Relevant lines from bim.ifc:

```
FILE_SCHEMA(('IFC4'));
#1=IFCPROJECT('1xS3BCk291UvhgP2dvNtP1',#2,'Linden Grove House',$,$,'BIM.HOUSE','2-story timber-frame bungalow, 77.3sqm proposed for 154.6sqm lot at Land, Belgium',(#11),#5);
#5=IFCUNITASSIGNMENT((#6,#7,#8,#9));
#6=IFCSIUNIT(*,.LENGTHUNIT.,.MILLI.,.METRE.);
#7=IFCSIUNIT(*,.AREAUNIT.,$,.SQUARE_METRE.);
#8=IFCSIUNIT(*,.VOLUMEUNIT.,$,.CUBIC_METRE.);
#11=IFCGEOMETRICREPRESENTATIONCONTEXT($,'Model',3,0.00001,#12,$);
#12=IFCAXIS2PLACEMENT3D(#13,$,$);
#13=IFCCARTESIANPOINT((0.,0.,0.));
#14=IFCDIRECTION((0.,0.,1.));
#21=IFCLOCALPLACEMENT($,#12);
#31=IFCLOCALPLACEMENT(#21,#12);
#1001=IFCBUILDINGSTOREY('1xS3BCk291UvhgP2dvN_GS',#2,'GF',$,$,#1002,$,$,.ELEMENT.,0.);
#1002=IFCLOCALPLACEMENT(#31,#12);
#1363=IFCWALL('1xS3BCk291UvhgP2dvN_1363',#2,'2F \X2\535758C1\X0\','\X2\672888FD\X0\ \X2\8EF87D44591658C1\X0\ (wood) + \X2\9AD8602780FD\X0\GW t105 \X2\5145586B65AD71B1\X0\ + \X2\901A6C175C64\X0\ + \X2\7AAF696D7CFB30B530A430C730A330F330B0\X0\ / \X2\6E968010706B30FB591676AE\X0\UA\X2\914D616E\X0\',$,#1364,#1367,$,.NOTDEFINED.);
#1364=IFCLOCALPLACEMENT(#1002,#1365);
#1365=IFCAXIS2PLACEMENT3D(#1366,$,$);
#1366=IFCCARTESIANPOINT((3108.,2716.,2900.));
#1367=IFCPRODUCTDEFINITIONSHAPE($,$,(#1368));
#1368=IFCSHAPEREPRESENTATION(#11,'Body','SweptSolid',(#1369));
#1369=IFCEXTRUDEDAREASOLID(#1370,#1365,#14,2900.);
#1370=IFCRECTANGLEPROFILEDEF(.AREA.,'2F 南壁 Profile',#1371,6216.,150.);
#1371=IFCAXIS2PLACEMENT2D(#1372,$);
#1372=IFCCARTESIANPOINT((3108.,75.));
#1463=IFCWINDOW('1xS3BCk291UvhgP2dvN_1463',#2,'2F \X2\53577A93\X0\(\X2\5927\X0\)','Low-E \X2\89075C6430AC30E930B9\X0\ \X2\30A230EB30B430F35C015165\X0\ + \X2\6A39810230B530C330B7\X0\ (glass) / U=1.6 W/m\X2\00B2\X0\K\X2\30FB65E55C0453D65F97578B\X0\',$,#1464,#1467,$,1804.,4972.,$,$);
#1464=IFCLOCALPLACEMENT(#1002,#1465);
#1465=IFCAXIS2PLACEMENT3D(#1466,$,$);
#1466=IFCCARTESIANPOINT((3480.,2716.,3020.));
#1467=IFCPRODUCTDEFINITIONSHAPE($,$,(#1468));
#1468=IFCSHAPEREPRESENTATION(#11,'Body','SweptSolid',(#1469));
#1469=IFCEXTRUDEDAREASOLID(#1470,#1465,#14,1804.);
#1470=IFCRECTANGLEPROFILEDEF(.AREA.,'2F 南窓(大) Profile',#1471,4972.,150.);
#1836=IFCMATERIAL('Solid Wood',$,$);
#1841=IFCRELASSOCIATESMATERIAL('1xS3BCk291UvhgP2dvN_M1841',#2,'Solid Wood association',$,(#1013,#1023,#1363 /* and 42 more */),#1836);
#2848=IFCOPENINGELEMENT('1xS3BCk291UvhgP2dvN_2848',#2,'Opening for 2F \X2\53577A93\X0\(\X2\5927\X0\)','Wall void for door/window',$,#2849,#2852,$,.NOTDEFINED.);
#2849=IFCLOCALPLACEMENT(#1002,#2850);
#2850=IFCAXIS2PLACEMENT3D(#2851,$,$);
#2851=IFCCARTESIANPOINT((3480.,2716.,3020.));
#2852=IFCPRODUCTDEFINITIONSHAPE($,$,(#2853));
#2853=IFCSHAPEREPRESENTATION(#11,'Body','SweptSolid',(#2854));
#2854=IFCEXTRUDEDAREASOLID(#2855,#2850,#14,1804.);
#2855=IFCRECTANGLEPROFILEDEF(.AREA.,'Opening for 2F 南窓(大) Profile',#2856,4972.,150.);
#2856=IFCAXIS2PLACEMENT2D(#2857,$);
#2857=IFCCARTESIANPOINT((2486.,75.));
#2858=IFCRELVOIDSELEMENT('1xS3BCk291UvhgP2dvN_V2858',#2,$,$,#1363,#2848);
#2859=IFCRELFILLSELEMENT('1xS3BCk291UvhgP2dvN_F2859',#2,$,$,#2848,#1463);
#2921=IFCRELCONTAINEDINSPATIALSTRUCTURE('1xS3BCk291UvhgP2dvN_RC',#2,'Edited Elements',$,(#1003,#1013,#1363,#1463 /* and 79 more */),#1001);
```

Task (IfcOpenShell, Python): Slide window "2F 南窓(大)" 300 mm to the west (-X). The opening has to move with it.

```python
import ifcopenshell
import ifcopenshell.api.geometry
import ifcopenshell.util.placement

model = ifcopenshell.open("bim.ifc")

window = model.by_guid("1xS3BCk291UvhgP2dvN_1463")
opening = window.FillsVoids[0].RelatingOpeningElement
wall = opening.VoidsElements[0].RelatingBuildingElement

wall_matrix = ifcopenshell.util.placement.get_local_placement(wall.ObjectPlacement)
shift = wall_matrix[:3, 0] * -300.0
before = ifcopenshell.util.placement.get_local_placement(window.ObjectPlacement)[:3, 3].copy()

# The window is not placed relative to its opening, so move both.
for product in (opening, window):
    matrix = ifcopenshell.util.placement.get_local_placement(product.ObjectPlacement)
    matrix[:3, 3] += shift
    ifcopenshell.api.geometry.edit_object_placement(model, product=product, matrix=matrix, is_si=False)

after = ifcopenshell.util.placement.get_local_placement(window.ObjectPlacement)[:3, 3]
print("window moved by", (after - before).round(3) + 0.0)

model.write("bim_v2.ifc")
```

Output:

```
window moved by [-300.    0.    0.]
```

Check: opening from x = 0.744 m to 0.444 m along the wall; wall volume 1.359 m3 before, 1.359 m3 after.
